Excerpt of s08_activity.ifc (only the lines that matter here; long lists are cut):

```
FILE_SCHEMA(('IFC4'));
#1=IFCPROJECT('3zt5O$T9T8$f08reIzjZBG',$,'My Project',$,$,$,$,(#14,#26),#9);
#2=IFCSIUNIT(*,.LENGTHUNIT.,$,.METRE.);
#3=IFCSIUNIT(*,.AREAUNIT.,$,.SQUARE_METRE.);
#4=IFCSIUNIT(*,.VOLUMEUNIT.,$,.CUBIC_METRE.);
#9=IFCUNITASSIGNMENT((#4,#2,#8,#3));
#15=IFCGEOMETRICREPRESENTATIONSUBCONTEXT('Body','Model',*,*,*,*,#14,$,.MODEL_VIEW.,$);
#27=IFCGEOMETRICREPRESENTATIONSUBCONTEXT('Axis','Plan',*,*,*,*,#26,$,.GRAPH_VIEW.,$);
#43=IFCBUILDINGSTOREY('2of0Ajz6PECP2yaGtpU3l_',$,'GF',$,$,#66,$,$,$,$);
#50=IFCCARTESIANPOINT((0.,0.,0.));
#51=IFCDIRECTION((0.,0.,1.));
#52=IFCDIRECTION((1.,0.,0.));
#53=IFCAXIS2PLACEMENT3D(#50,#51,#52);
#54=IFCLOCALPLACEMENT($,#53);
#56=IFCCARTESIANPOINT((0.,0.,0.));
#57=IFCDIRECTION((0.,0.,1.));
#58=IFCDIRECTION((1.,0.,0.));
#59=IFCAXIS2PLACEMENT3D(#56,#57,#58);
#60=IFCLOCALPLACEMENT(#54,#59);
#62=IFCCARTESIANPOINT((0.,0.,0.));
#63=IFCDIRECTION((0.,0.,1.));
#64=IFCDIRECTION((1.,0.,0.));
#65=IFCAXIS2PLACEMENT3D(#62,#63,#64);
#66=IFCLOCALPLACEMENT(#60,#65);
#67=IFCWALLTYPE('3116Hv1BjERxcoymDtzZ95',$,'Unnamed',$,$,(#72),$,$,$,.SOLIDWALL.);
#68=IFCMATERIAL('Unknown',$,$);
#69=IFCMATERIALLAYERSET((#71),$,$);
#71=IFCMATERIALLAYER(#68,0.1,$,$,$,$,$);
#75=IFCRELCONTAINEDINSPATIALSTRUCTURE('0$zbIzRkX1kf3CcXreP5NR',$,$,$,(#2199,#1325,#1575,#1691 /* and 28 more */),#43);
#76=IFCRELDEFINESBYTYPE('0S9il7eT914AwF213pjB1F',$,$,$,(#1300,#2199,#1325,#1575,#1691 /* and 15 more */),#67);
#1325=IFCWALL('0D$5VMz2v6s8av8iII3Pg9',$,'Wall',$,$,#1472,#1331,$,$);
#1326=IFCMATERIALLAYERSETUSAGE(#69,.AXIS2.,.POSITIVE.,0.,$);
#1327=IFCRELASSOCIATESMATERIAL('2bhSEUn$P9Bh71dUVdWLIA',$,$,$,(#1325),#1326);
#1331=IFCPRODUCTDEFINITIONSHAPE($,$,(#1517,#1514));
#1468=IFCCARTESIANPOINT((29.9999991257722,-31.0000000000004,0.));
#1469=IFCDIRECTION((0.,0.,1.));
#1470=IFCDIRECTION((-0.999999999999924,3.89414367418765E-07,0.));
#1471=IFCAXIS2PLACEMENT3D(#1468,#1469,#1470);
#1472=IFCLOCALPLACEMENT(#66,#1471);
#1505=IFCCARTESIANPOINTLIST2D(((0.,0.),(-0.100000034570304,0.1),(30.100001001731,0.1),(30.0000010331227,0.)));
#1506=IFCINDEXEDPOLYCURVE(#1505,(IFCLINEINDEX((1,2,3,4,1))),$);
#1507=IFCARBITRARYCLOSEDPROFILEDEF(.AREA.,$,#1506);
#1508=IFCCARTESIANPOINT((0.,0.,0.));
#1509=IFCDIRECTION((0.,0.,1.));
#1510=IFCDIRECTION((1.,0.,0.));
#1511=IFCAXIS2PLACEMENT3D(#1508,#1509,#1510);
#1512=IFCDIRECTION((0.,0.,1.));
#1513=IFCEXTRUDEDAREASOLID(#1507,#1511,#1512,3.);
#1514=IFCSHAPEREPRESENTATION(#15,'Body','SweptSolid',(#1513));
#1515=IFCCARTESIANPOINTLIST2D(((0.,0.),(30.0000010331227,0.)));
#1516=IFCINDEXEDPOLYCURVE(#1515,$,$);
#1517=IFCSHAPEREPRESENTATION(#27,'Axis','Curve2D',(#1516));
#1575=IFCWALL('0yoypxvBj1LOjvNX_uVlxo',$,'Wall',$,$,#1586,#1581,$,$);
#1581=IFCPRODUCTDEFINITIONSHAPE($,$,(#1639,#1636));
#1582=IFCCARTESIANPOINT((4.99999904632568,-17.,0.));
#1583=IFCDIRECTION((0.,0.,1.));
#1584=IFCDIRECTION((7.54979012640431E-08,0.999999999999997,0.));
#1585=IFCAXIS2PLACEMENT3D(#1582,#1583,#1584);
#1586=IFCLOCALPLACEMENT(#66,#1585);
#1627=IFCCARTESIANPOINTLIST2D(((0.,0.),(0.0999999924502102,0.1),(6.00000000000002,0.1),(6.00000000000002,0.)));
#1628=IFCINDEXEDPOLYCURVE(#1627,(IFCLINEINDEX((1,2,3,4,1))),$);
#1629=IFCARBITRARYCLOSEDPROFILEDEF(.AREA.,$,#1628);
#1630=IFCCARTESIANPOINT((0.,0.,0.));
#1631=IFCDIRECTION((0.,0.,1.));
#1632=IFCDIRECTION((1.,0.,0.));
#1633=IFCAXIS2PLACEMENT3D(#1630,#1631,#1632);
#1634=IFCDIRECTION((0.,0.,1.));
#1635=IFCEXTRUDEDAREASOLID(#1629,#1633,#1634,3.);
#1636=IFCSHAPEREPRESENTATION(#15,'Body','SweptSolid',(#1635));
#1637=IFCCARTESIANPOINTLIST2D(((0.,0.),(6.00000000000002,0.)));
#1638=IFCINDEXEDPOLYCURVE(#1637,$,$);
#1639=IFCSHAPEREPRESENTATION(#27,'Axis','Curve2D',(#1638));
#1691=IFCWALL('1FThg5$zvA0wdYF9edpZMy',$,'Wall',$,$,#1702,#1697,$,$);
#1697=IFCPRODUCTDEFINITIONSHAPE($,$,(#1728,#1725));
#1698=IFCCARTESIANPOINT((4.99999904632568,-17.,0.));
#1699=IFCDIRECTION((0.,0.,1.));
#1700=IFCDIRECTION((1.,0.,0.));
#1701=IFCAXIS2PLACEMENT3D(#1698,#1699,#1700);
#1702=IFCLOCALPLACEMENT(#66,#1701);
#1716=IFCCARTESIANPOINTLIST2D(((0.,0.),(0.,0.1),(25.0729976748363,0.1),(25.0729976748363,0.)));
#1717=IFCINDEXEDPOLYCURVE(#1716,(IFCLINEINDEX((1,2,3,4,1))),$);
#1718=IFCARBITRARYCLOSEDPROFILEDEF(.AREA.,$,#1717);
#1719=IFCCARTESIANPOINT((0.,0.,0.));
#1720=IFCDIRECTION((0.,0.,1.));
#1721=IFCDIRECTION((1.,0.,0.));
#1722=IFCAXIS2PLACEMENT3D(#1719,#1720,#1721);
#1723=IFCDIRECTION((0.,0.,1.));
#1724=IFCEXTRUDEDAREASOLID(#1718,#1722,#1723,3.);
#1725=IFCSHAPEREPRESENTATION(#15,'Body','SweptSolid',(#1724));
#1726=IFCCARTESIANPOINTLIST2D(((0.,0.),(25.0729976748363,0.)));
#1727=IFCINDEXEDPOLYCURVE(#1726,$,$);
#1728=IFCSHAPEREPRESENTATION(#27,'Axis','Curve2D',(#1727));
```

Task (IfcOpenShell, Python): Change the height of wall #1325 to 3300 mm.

```python
import ifcopenshell
import ifcopenshell.geom
import ifcopenshell.util.representation
import ifcopenshell.util.shape
import ifcopenshell.util.unit

model = ifcopenshell.open("s08_activity.ifc")
unit_scale = ifcopenshell.util.unit.calculate_unit_scale(model)
settings = ifcopenshell.geom.settings()


def volume(element):
    """Net volume in cubic metres, openings subtracted."""
    shape = ifcopenshell.geom.create_shape(settings, element)
    return ifcopenshell.util.shape.get_volume(shape.geometry)


wall = model.by_guid("0D$5VMz2v6s8av8iII3Pg9")
before = volume(wall)

body = ifcopenshell.util.representation.get_representation(wall, "Model", "Body")
solid = body.Items[0]
old_height = solid.Depth
solid.Depth = 3.3 / unit_scale
after = volume(wall)

print(f"height {old_height:g} -> {solid.Depth:g}, volume {before:.3f} -> {after:.3f} m3")

model.write("s08_activity-out.ifc")
```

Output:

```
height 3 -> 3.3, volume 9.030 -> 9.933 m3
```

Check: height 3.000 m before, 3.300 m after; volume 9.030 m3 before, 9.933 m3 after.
